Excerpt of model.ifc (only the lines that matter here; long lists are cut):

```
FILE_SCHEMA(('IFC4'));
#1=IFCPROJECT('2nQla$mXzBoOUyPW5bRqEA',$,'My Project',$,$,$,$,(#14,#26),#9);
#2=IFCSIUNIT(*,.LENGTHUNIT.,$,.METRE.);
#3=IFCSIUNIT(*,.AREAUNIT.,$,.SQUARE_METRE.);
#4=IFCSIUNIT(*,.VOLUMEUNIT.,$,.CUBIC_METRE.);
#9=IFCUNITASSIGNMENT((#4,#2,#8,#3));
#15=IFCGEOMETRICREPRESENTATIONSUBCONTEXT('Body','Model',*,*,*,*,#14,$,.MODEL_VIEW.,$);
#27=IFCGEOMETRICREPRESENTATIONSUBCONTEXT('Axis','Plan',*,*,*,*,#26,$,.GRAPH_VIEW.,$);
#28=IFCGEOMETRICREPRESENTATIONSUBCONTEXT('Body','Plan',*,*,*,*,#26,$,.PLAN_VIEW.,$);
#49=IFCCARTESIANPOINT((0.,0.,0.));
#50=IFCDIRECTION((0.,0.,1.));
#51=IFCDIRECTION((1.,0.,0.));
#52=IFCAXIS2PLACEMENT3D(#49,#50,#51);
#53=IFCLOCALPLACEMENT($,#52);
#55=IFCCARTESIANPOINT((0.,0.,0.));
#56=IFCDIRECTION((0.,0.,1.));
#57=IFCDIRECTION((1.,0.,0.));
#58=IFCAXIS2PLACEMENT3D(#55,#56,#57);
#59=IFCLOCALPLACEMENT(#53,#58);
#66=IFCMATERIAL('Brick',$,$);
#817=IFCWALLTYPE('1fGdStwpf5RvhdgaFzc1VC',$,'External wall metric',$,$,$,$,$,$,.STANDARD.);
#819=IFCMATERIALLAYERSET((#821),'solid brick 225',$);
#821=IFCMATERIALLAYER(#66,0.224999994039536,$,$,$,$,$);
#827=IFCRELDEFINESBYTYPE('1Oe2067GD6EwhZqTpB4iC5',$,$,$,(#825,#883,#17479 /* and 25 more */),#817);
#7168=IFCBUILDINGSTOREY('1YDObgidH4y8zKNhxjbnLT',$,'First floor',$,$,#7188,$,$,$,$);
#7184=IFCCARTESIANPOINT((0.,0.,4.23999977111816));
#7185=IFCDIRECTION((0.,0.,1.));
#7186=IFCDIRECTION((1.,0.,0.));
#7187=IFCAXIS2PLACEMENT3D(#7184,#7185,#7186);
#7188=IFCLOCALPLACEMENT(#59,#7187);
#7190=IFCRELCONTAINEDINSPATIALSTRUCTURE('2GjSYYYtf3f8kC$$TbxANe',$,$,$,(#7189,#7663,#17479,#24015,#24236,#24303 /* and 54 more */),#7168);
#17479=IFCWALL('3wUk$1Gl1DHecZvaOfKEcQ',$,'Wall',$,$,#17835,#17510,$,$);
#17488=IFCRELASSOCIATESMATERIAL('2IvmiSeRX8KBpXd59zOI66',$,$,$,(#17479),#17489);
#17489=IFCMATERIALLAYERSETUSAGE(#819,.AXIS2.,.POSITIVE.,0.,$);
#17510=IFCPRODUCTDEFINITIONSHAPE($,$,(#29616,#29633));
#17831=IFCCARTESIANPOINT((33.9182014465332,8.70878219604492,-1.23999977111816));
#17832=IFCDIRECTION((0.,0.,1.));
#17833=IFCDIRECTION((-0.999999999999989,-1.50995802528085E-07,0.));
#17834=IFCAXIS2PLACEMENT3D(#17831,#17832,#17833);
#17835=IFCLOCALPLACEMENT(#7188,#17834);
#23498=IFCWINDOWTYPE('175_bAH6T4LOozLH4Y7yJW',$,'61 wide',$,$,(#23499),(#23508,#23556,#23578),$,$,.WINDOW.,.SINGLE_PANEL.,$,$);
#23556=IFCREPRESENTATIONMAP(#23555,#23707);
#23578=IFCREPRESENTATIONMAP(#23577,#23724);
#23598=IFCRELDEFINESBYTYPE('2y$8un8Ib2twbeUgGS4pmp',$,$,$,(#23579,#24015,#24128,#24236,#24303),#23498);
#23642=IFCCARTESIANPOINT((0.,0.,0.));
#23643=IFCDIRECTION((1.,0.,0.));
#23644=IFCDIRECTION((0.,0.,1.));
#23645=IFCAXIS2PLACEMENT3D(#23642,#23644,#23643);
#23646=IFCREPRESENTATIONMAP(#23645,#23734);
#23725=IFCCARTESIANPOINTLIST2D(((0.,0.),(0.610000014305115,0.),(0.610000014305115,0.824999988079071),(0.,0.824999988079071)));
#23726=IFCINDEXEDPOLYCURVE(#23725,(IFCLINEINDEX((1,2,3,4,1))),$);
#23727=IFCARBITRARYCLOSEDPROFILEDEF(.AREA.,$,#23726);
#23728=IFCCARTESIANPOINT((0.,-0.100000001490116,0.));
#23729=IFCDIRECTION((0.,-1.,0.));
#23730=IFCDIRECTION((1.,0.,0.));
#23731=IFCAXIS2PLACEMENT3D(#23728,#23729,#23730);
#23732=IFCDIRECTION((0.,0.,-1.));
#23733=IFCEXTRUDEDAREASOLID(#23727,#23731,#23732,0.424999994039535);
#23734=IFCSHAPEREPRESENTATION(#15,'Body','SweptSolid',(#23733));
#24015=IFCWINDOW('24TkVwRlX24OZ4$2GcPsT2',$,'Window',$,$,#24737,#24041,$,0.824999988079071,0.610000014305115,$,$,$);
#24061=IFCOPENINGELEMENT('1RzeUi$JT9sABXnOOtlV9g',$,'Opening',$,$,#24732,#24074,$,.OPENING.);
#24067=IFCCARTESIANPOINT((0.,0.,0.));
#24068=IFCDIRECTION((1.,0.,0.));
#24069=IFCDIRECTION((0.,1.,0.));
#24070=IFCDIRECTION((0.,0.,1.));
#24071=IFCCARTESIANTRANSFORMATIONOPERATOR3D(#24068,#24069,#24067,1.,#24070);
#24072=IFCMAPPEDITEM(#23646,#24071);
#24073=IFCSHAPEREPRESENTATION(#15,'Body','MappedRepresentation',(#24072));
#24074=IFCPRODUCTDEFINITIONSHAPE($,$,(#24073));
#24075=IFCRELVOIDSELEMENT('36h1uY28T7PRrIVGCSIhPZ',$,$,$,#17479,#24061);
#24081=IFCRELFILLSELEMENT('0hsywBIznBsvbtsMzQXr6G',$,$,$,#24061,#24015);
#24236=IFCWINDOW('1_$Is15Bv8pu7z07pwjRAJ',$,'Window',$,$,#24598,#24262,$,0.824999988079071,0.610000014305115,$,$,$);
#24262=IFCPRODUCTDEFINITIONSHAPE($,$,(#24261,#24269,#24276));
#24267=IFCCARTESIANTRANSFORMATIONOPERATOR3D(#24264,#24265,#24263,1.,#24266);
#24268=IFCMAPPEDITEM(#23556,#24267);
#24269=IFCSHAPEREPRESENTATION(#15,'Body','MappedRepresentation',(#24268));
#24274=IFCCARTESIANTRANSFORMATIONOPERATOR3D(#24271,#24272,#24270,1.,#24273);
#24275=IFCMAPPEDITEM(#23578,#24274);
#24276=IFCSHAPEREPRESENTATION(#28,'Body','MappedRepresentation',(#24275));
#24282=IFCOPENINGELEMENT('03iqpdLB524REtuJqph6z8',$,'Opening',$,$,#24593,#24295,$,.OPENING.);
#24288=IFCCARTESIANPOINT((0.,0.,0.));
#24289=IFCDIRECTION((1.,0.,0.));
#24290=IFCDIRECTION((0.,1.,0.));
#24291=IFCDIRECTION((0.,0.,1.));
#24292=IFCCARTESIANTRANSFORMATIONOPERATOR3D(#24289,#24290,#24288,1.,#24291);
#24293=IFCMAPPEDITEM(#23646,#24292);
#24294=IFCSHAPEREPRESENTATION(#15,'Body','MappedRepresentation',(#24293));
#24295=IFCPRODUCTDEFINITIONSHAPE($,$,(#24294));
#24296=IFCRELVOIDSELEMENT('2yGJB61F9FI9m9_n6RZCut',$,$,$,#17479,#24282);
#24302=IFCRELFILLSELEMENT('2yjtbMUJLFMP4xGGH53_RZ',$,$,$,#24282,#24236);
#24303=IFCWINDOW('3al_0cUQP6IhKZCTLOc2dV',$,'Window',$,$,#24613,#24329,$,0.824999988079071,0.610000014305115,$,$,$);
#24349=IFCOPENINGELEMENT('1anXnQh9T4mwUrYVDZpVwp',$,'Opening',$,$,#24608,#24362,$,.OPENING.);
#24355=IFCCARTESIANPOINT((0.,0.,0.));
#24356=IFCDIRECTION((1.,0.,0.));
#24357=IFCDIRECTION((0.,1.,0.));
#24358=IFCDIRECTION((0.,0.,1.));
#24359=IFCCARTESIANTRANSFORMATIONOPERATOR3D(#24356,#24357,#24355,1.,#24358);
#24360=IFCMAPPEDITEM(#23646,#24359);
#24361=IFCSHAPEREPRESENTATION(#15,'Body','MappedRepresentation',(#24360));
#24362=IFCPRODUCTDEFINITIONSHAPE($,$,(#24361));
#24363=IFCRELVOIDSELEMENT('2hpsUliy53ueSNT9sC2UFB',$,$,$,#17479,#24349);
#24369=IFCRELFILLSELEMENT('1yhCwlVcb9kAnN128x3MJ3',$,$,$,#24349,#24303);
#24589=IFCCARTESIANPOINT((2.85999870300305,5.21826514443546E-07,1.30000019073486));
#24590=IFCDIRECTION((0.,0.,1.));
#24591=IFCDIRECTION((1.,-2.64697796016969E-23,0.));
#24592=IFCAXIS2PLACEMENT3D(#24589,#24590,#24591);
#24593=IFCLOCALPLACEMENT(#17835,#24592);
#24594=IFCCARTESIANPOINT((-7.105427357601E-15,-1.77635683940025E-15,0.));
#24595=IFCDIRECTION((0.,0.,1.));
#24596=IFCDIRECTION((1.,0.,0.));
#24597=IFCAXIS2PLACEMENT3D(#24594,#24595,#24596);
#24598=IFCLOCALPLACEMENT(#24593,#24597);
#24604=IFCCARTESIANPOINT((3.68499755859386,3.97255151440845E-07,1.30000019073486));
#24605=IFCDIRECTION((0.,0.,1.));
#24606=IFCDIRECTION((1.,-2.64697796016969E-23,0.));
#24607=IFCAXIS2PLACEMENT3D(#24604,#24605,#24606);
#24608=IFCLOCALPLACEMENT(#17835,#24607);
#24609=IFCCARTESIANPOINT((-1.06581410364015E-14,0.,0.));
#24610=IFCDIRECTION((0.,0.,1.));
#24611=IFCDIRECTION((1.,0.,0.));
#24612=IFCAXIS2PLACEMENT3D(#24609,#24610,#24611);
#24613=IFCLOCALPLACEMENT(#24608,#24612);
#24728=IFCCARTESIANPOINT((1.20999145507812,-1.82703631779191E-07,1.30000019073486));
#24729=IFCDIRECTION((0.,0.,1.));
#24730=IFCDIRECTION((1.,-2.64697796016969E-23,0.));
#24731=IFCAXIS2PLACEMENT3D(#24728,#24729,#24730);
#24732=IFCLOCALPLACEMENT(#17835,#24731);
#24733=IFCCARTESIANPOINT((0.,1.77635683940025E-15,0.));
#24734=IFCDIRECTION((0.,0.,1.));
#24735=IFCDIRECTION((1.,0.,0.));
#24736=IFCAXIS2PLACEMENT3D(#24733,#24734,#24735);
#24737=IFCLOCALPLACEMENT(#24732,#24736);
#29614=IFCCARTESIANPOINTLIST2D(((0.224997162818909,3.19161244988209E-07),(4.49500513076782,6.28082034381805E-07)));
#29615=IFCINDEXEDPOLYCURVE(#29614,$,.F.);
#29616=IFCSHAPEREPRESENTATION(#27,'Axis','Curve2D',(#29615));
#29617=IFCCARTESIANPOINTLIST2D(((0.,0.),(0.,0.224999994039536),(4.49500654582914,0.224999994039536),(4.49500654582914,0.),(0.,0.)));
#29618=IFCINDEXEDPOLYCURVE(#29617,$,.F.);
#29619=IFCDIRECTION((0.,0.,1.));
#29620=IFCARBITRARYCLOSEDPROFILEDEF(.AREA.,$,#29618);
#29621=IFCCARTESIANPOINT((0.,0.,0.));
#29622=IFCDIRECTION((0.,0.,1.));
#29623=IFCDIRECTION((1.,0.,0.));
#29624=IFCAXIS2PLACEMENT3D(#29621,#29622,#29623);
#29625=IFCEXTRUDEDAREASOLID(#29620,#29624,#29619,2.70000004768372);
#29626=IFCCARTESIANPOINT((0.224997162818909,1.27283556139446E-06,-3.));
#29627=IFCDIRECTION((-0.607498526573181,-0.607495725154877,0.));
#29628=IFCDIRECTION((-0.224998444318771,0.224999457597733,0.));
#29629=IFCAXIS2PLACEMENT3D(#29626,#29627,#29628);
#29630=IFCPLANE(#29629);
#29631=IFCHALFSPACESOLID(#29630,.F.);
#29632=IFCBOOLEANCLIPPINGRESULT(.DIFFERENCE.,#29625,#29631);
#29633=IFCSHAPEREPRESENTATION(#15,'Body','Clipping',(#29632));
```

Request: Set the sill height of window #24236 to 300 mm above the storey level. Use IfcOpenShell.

```python
import numpy as np
import ifcopenshell
import ifcopenshell.api.geometry
import ifcopenshell.geom
import ifcopenshell.util.element
import ifcopenshell.util.placement
import ifcopenshell.util.shape
import ifcopenshell.util.unit

model = ifcopenshell.open("model.ifc")
unit_scale = ifcopenshell.util.unit.calculate_unit_scale(model)

window = model.by_id(24236)
opening = window.FillsVoids[0].RelatingOpeningElement
storey = ifcopenshell.util.element.get_container(window, ifc_class="IfcBuildingStorey")
level = ifcopenshell.util.placement.get_local_placement(storey.ObjectPlacement)[2, 3]

# The opening's origin need not be at the sill, so measure its lowest point.
shape = ifcopenshell.geom.create_shape(ifcopenshell.geom.settings(), opening)
bottom = ifcopenshell.util.shape.get_shape_bottom_elevation(shape, shape.geometry) / unit_scale
dz = level + 0.3 - bottom

shift = np.array([0.0, 0.0, dz])
# The window is placed relative to its opening, so it follows when the opening moves.
matrix = ifcopenshell.util.placement.get_local_placement(opening.ObjectPlacement)
matrix[:3, 3] += shift
ifcopenshell.api.geometry.edit_object_placement(
    model, product=opening, matrix=matrix, is_si=False, should_transform_children=True
)

print(f"moved by {dz * unit_scale:+.3f} m")

model.write("model_v2.ifc")
```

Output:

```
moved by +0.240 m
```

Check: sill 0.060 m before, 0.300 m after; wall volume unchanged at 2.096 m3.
